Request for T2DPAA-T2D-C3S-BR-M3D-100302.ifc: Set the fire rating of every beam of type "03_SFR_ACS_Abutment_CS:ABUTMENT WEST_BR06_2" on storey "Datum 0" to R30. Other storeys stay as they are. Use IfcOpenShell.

First a look at what the model holds.

```python
import ifcopenshell
import ifcopenshell.util.element

model = ifcopenshell.open("T2DPAA-T2D-C3S-BR-M3D-100302.ifc")
print(model.schema)
storey = next(s for s in model.by_type("IfcBuildingStorey") if s.Name == "Datum 0")
beams = [e for e in ifcopenshell.util.element.get_decomposition(storey) if e.is_a("IfcBeam")]
seen = {}
for e in beams:
    element_type = ifcopenshell.util.element.get_type(e)
    key = (element_type.Name if element_type != e and element_type else None, ifcopenshell.util.element.get_pset(e, "Pset_BeamCommon", "FireRating"))
    seen[key] = seen.get(key, 0) + 1
for (name, value), count in sorted(seen.items(), key=str):
    print(count, "x", name, "|", value)
```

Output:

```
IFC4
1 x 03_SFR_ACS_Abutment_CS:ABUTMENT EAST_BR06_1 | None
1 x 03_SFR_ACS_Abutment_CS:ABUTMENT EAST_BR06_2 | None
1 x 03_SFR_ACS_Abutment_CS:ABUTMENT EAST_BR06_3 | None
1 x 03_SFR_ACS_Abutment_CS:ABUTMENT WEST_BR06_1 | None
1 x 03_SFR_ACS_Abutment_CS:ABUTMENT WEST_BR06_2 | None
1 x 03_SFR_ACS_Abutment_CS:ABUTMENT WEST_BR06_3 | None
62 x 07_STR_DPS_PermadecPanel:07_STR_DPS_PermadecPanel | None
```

```python
import ifcopenshell
import ifcopenshell.api.pset
import ifcopenshell.util.element

model = ifcopenshell.open("T2DPAA-T2D-C3S-BR-M3D-100302.ifc")

storey = next(s for s in model.by_type("IfcBuildingStorey") if s.Name == "Datum 0")
beams = [e for e in ifcopenshell.util.element.get_decomposition(storey) if e.is_a("IfcBeam")]

count = 0
for e in beams:
    element_type = ifcopenshell.util.element.get_type(e)
    if element_type in (None, e) or element_type.Name != "03_SFR_ACS_Abutment_CS:ABUTMENT WEST_BR06_2":
        continue
    # add_pset returns the element's existing set when there is one.
    pset = ifcopenshell.api.pset.add_pset(model, product=e, name="Pset_BeamCommon")
    ifcopenshell.api.pset.edit_pset(model, pset=pset, properties={"FireRating": "R30"})
    count += 1

print(count, "beams updated")

model.write("T2DPAA-T2D-C3S-BR-M3D-100302_rev.ifc")
```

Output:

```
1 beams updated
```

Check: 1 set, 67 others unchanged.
